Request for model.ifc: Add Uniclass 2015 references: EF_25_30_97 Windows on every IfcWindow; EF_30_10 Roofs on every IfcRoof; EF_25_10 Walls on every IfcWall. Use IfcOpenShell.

First a look at what the model holds.

```python
import ifcopenshell

model = ifcopenshell.open("model.ifc")
print(model.schema)
print("classifications:", [c.Name for c in model.by_type("IfcClassification")])
for ifc_class in ("IfcDoor", "IfcRoof", "IfcStair", "IfcWall", "IfcWindow"):
    print(ifc_class, len(model.by_type(ifc_class)))
```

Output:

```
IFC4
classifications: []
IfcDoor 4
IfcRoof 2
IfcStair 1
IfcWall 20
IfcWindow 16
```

```python
import ifcopenshell
import ifcopenshell.api.classification

model = ifcopenshell.open("model.ifc")

system = ifcopenshell.api.classification.add_classification(model, classification="Uniclass 2015")

codes = {
    "IfcWindow": ("EF_25_30_97", "Windows"),
    "IfcRoof": ("EF_30_10", "Roofs"),
    "IfcWall": ("EF_25_10", "Walls"),
}
for ifc_class, (code, name) in codes.items():
    products = model.by_type(ifc_class)
    ifcopenshell.api.classification.add_reference(
        model, products=products, classification=system, identification=code, name=name
    )
    print(code, len(products))

model.write("model_v2.ifc")
```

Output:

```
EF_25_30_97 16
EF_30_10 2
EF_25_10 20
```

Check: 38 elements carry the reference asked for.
